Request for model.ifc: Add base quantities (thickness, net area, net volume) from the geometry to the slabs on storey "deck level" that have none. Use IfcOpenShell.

First a look at what the model holds.

```python
import ifcopenshell
import ifcopenshell.util.element
import ifcopenshell.util.unit

model = ifcopenshell.open("model.ifc")
print(model.schema)
for unit_type in ("LENGTHUNIT", "AREAUNIT", "VOLUMEUNIT"):
    print(unit_type, ifcopenshell.util.unit.calculate_unit_scale(model, unit_type))
storey = next(s for s in model.by_type("IfcBuildingStorey") if s.Name == "deck level")
slabs = [e for e in ifcopenshell.util.element.get_decomposition(storey) if e.is_a("IfcSlab")]
for e in sorted(slabs, key=lambda e: e.id()):
    print(e.id(), e.is_a(), e.Name, list(ifcopenshell.util.element.get_psets(e, qtos_only=True)), sep=" | ")
```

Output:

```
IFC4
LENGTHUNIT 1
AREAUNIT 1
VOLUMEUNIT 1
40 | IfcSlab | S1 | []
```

```python
import ifcopenshell
import ifcopenshell.api.pset
import ifcopenshell.geom
import ifcopenshell.util.element
import ifcopenshell.util.shape
import ifcopenshell.util.unit

model = ifcopenshell.open("model.ifc")
unit_scale = ifcopenshell.util.unit.calculate_unit_scale(model)
area_scale = ifcopenshell.util.unit.calculate_unit_scale(model, "AREAUNIT")
volume_scale = ifcopenshell.util.unit.calculate_unit_scale(model, "VOLUMEUNIT")
settings = ifcopenshell.geom.settings()

storey = next(s for s in model.by_type("IfcBuildingStorey") if s.Name == "deck level")
slabs = [e for e in ifcopenshell.util.element.get_decomposition(storey) if e.is_a("IfcSlab")]

for e in sorted(slabs, key=lambda e: e.id()):
    if ifcopenshell.util.element.get_psets(e, qtos_only=True, should_inherit=False):
        continue
    # Geometry comes back in metres, in the element's own axes.
    shape = ifcopenshell.geom.create_shape(settings, e)
    values = {
        "Width": ifcopenshell.util.shape.get_z(shape.geometry) / unit_scale,
        "NetArea": ifcopenshell.util.shape.get_footprint_area(shape.geometry) / area_scale,
        "NetVolume": ifcopenshell.util.shape.get_volume(shape.geometry) / volume_scale,
    }
    qto = ifcopenshell.api.pset.add_qto(model, product=e, name="Qto_SlabBaseQuantities")
    ifcopenshell.api.pset.edit_qto(model, qto=qto, properties=values)
    print(e.id(), {k: round(v, 3) for k, v in values.items()})

model.write("model_rev.ifc")
```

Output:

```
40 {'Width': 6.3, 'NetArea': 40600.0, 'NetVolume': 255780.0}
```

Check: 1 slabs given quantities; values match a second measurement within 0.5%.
